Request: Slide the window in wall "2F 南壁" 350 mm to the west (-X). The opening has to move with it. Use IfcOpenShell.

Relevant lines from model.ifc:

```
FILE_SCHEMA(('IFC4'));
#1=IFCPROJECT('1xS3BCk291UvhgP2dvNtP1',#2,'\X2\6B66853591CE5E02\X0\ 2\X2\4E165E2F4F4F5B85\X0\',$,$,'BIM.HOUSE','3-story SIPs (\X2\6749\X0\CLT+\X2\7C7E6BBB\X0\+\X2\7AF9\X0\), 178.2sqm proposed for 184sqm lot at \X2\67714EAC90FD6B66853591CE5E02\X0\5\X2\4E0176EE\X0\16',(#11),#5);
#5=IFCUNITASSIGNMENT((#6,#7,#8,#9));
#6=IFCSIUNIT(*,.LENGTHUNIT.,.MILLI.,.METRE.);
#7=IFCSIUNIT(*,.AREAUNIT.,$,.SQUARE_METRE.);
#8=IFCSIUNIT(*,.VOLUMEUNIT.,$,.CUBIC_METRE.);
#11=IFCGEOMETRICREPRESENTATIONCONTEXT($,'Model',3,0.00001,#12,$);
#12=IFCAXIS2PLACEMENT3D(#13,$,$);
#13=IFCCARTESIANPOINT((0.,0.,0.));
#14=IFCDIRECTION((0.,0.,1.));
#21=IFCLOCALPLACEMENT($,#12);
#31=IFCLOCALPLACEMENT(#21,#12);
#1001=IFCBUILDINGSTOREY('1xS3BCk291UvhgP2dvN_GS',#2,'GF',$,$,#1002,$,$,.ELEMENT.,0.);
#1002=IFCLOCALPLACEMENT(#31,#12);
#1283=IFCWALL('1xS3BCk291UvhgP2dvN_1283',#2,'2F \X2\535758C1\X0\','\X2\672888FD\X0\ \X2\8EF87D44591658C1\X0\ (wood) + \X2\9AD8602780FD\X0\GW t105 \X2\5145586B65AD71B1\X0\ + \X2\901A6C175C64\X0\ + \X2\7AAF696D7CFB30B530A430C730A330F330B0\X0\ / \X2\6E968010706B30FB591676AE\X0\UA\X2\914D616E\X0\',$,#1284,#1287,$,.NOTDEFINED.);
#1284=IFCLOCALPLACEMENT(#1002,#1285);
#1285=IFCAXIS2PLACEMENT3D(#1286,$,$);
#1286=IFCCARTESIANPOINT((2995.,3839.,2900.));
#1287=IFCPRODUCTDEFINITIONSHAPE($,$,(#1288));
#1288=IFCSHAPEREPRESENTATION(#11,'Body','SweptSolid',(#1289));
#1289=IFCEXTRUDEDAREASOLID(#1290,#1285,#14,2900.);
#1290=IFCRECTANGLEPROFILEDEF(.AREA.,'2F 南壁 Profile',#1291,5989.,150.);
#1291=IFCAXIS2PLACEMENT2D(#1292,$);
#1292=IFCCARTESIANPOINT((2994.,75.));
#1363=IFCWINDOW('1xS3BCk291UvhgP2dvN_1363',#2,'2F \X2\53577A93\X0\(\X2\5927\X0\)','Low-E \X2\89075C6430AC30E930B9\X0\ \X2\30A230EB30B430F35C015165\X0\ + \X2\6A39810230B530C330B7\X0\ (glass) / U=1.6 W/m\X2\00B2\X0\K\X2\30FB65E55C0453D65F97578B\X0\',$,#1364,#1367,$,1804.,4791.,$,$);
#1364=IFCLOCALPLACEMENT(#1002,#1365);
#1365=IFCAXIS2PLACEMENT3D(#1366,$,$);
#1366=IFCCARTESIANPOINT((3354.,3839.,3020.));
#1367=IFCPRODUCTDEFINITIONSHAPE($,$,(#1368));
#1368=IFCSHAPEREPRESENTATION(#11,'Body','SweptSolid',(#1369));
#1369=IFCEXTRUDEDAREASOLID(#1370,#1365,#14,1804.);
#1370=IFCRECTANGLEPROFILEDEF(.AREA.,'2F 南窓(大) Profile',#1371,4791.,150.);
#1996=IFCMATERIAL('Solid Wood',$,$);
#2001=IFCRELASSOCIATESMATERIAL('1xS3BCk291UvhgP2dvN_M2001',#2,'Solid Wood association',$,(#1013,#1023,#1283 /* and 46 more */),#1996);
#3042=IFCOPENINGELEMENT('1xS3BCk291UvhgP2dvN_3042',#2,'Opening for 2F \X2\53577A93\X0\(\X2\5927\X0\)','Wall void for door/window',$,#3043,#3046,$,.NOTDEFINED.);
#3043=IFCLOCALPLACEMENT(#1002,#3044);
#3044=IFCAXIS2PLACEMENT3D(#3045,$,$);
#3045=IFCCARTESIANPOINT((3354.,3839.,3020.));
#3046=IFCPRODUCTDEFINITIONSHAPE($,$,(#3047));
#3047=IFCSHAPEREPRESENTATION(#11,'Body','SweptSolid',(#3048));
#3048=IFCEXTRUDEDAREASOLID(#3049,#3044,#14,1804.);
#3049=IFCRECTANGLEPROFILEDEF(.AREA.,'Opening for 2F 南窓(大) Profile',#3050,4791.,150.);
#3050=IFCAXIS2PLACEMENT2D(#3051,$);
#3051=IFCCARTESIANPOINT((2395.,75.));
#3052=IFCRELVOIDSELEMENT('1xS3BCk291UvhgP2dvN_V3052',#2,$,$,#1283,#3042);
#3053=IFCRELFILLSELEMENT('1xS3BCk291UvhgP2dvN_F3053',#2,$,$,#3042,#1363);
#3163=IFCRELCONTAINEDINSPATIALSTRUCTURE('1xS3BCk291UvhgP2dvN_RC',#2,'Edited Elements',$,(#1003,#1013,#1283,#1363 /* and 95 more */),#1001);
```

```python
import ifcopenshell
import ifcopenshell.api.geometry
import ifcopenshell.util.placement
import ifcopenshell.util.unit

model = ifcopenshell.open("model.ifc")
unit_scale = ifcopenshell.util.unit.calculate_unit_scale(model)

window = model.by_id(1363)
opening = window.FillsVoids[0].RelatingOpeningElement
wall = opening.VoidsElements[0].RelatingBuildingElement

wall_matrix = ifcopenshell.util.placement.get_local_placement(wall.ObjectPlacement)
shift = wall_matrix[:3, 0] * -0.35 / unit_scale
before = ifcopenshell.util.placement.get_local_placement(window.ObjectPlacement)[:3, 3].copy()

# The window is not placed relative to its opening, so move both.
for product in (opening, window):
    matrix = ifcopenshell.util.placement.get_local_placement(product.ObjectPlacement)
    matrix[:3, 3] += shift
    ifcopenshell.api.geometry.edit_object_placement(model, product=product, matrix=matrix, is_si=False)

after = ifcopenshell.util.placement.get_local_placement(window.ObjectPlacement)[:3, 3]
print("window moved by", (after - before).round(3) + 0.0)

model.write("model_updated.ifc")
```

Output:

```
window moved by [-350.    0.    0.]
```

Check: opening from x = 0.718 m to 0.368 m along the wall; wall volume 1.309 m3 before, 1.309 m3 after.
